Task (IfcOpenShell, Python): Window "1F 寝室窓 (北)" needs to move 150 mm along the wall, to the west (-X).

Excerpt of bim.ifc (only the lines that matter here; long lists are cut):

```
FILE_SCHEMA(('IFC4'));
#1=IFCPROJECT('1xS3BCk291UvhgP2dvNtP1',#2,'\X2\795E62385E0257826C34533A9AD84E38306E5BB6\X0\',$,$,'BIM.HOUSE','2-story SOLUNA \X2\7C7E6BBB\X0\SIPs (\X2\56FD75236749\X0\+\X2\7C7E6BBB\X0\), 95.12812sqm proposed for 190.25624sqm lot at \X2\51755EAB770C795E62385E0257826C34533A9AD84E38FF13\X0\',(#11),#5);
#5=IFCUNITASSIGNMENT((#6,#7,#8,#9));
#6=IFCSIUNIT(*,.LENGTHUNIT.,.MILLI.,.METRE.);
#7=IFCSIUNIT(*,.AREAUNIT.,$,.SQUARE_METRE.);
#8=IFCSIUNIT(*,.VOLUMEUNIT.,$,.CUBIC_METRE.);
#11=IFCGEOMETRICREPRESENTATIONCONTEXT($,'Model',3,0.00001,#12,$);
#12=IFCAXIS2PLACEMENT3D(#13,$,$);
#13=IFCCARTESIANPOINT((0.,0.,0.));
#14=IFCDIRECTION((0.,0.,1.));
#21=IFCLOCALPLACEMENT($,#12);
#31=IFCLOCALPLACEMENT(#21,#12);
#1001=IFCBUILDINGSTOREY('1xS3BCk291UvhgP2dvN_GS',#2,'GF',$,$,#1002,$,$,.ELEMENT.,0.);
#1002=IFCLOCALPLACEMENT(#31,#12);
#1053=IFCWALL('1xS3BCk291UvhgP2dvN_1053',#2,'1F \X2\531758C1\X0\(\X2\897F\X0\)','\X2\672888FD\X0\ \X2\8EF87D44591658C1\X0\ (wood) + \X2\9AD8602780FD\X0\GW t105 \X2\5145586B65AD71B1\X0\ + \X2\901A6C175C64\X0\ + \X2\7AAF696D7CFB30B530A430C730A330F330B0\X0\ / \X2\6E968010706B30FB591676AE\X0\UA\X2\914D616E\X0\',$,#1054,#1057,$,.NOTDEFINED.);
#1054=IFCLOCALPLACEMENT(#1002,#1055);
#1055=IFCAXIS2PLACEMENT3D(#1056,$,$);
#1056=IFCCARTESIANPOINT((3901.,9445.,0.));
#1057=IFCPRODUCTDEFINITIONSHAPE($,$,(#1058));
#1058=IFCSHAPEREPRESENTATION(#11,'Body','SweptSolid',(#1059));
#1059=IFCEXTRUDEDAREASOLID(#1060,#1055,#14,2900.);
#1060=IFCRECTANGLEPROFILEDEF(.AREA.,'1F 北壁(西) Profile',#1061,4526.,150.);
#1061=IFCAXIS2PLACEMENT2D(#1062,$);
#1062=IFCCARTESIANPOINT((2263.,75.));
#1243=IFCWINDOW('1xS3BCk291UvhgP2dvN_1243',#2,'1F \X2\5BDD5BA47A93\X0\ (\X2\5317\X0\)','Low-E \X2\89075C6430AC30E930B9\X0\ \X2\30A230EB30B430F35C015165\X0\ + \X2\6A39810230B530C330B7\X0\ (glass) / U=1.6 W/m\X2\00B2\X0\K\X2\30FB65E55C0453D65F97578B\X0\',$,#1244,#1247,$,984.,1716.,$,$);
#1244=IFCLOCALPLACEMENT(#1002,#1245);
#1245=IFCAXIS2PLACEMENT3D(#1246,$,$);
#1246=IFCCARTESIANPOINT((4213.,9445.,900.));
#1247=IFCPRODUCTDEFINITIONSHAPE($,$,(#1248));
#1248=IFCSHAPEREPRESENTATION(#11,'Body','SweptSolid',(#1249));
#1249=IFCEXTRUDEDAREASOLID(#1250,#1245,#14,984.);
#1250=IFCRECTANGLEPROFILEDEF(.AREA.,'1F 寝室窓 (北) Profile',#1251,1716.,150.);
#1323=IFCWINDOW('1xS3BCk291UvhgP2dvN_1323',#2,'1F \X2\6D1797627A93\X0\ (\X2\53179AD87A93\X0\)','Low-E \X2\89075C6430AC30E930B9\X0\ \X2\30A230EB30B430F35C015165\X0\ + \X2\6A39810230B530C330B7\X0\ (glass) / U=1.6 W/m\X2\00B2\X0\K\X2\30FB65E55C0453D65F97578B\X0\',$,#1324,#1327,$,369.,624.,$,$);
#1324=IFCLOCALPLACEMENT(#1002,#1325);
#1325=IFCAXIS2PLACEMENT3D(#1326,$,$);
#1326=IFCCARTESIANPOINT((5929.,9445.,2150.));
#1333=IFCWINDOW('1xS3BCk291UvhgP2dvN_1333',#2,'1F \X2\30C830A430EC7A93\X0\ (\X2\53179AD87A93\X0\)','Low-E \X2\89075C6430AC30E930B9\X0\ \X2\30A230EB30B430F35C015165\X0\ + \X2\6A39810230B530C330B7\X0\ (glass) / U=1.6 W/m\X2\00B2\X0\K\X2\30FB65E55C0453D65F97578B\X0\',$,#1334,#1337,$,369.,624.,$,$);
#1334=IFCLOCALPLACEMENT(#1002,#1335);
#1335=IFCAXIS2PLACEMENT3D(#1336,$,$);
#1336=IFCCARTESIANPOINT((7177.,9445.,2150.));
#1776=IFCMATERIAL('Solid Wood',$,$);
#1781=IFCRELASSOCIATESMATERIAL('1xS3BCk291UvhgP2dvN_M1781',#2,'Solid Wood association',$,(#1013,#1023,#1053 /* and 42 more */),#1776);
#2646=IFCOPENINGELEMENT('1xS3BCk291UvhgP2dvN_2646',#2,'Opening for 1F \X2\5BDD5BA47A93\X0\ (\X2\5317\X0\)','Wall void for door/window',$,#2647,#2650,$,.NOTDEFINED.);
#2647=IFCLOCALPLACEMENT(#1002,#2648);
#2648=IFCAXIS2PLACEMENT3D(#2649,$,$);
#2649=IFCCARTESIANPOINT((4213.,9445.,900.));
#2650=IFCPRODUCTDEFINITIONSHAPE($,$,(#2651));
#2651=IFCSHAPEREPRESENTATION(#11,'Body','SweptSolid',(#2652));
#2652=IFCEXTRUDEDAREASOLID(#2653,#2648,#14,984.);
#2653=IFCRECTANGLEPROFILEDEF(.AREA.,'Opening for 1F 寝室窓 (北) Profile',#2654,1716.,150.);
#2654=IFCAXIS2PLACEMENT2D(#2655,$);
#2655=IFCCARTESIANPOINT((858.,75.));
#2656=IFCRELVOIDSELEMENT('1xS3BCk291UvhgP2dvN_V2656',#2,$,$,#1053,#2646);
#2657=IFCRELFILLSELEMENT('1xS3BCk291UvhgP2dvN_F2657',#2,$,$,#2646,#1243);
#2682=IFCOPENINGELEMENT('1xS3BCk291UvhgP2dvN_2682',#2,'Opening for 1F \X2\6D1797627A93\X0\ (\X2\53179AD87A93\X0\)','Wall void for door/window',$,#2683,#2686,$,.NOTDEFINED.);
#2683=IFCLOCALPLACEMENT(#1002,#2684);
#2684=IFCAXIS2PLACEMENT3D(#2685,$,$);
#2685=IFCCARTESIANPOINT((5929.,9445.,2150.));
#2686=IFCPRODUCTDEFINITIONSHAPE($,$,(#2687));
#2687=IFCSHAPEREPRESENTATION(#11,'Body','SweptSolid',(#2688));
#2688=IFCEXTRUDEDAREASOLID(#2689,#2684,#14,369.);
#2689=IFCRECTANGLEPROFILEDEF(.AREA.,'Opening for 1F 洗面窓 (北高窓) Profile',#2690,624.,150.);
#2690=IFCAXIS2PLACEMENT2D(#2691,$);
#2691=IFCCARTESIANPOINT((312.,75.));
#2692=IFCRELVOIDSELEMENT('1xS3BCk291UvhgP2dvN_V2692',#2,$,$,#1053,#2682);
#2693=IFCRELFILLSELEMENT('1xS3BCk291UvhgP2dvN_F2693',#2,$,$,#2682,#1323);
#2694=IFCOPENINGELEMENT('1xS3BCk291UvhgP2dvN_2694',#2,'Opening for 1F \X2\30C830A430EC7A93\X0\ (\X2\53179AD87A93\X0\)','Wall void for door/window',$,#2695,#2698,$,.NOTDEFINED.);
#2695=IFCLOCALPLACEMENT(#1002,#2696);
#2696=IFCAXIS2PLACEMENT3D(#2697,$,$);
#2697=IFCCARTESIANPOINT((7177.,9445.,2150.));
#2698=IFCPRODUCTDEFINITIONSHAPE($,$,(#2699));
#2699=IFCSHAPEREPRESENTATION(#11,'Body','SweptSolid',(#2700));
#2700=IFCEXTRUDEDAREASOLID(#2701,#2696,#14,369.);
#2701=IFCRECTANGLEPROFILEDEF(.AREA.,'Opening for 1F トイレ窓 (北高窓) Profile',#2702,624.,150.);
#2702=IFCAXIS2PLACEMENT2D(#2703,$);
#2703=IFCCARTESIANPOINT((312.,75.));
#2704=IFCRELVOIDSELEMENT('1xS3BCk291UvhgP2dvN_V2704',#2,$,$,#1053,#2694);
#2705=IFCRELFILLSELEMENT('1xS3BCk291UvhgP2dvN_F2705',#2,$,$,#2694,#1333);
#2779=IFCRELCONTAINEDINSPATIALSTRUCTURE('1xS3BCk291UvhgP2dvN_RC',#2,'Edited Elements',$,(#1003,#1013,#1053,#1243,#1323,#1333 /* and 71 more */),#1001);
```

```python
import ifcopenshell
import ifcopenshell.api.geometry
import ifcopenshell.util.placement

model = ifcopenshell.open("bim.ifc")

window = model.by_guid("1xS3BCk291UvhgP2dvN_1243")
opening = window.FillsVoids[0].RelatingOpeningElement
wall = opening.VoidsElements[0].RelatingBuildingElement

wall_matrix = ifcopenshell.util.placement.get_local_placement(wall.ObjectPlacement)
shift = wall_matrix[:3, 0] * -150.0
before = ifcopenshell.util.placement.get_local_placement(window.ObjectPlacement)[:3, 3].copy()

# The window is not placed relative to its opening, so move both.
for product in (opening, window):
    matrix = ifcopenshell.util.placement.get_local_placement(product.ObjectPlacement)
    matrix[:3, 3] += shift
    ifcopenshell.api.geometry.edit_object_placement(model, product=product, matrix=matrix, is_si=False)

after = ifcopenshell.util.placement.get_local_placement(window.ObjectPlacement)[:3, 3]
print("window moved by", (after - before).round(3) + 0.0)

model.write("bim_edited.ifc")
```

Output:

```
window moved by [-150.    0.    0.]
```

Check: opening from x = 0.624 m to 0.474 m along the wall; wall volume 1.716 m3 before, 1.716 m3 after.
